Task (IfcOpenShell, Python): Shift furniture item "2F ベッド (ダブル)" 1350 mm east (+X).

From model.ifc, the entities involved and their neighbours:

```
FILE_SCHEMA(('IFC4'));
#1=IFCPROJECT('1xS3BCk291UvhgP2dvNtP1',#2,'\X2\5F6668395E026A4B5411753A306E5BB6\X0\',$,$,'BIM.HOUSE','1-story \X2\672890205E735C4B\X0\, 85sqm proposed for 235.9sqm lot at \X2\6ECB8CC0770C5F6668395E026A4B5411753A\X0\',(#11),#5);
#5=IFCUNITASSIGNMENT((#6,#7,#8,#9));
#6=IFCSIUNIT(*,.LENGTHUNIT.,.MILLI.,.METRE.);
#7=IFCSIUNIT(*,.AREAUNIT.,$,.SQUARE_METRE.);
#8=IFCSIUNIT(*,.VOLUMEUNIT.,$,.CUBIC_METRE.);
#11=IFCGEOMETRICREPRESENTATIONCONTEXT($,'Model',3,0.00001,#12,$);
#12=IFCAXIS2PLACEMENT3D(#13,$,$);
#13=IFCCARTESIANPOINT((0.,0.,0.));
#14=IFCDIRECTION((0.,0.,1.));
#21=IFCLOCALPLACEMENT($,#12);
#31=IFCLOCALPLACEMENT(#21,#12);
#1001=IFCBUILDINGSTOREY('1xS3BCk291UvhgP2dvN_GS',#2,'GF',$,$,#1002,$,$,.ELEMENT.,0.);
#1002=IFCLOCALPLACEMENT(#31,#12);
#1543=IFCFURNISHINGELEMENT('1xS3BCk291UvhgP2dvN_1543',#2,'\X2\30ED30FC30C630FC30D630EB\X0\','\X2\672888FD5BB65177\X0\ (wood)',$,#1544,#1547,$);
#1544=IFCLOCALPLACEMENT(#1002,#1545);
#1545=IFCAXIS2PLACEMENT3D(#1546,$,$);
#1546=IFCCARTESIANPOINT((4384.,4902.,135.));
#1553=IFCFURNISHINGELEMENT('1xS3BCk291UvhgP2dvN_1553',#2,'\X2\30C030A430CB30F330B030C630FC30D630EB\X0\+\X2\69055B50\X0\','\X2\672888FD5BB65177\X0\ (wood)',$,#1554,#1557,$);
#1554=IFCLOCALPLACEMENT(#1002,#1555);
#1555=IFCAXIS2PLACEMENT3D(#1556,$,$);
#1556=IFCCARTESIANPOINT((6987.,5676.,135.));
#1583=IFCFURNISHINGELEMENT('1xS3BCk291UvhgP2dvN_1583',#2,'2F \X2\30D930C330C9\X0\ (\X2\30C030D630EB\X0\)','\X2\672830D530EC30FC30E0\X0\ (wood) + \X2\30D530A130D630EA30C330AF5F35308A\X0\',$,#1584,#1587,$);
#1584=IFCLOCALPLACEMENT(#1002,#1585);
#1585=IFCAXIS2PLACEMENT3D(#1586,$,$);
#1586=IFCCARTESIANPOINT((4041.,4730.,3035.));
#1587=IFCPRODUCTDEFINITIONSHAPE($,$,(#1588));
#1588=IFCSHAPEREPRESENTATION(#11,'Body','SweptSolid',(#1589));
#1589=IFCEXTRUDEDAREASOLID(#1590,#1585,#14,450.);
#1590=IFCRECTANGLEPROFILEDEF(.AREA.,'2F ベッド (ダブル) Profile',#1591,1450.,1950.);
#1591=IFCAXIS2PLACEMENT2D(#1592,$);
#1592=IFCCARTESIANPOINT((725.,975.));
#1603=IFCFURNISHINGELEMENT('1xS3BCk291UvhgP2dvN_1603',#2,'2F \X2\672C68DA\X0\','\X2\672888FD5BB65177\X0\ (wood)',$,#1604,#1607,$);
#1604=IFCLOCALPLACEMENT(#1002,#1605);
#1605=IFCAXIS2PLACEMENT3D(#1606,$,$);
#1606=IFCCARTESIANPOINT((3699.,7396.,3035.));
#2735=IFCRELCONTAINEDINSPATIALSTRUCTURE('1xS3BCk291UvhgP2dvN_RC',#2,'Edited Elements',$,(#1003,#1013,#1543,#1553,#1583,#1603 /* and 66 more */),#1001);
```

```python
import ifcopenshell
import ifcopenshell.api.geometry
import ifcopenshell.util.placement

model = ifcopenshell.open("model.ifc")

item = model.by_id(1583)
matrix = ifcopenshell.util.placement.get_local_placement(item.ObjectPlacement)
matrix[0, 3] += 1350.0
ifcopenshell.api.geometry.edit_object_placement(model, product=item, matrix=matrix, is_si=False)

print(ifcopenshell.util.placement.get_local_placement(item.ObjectPlacement).round(3) + 0.0)

model.write("model_updated.ifc")
```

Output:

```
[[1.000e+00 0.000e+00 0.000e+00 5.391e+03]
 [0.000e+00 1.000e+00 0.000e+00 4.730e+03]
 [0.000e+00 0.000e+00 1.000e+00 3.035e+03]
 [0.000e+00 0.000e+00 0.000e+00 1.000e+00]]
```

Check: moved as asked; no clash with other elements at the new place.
